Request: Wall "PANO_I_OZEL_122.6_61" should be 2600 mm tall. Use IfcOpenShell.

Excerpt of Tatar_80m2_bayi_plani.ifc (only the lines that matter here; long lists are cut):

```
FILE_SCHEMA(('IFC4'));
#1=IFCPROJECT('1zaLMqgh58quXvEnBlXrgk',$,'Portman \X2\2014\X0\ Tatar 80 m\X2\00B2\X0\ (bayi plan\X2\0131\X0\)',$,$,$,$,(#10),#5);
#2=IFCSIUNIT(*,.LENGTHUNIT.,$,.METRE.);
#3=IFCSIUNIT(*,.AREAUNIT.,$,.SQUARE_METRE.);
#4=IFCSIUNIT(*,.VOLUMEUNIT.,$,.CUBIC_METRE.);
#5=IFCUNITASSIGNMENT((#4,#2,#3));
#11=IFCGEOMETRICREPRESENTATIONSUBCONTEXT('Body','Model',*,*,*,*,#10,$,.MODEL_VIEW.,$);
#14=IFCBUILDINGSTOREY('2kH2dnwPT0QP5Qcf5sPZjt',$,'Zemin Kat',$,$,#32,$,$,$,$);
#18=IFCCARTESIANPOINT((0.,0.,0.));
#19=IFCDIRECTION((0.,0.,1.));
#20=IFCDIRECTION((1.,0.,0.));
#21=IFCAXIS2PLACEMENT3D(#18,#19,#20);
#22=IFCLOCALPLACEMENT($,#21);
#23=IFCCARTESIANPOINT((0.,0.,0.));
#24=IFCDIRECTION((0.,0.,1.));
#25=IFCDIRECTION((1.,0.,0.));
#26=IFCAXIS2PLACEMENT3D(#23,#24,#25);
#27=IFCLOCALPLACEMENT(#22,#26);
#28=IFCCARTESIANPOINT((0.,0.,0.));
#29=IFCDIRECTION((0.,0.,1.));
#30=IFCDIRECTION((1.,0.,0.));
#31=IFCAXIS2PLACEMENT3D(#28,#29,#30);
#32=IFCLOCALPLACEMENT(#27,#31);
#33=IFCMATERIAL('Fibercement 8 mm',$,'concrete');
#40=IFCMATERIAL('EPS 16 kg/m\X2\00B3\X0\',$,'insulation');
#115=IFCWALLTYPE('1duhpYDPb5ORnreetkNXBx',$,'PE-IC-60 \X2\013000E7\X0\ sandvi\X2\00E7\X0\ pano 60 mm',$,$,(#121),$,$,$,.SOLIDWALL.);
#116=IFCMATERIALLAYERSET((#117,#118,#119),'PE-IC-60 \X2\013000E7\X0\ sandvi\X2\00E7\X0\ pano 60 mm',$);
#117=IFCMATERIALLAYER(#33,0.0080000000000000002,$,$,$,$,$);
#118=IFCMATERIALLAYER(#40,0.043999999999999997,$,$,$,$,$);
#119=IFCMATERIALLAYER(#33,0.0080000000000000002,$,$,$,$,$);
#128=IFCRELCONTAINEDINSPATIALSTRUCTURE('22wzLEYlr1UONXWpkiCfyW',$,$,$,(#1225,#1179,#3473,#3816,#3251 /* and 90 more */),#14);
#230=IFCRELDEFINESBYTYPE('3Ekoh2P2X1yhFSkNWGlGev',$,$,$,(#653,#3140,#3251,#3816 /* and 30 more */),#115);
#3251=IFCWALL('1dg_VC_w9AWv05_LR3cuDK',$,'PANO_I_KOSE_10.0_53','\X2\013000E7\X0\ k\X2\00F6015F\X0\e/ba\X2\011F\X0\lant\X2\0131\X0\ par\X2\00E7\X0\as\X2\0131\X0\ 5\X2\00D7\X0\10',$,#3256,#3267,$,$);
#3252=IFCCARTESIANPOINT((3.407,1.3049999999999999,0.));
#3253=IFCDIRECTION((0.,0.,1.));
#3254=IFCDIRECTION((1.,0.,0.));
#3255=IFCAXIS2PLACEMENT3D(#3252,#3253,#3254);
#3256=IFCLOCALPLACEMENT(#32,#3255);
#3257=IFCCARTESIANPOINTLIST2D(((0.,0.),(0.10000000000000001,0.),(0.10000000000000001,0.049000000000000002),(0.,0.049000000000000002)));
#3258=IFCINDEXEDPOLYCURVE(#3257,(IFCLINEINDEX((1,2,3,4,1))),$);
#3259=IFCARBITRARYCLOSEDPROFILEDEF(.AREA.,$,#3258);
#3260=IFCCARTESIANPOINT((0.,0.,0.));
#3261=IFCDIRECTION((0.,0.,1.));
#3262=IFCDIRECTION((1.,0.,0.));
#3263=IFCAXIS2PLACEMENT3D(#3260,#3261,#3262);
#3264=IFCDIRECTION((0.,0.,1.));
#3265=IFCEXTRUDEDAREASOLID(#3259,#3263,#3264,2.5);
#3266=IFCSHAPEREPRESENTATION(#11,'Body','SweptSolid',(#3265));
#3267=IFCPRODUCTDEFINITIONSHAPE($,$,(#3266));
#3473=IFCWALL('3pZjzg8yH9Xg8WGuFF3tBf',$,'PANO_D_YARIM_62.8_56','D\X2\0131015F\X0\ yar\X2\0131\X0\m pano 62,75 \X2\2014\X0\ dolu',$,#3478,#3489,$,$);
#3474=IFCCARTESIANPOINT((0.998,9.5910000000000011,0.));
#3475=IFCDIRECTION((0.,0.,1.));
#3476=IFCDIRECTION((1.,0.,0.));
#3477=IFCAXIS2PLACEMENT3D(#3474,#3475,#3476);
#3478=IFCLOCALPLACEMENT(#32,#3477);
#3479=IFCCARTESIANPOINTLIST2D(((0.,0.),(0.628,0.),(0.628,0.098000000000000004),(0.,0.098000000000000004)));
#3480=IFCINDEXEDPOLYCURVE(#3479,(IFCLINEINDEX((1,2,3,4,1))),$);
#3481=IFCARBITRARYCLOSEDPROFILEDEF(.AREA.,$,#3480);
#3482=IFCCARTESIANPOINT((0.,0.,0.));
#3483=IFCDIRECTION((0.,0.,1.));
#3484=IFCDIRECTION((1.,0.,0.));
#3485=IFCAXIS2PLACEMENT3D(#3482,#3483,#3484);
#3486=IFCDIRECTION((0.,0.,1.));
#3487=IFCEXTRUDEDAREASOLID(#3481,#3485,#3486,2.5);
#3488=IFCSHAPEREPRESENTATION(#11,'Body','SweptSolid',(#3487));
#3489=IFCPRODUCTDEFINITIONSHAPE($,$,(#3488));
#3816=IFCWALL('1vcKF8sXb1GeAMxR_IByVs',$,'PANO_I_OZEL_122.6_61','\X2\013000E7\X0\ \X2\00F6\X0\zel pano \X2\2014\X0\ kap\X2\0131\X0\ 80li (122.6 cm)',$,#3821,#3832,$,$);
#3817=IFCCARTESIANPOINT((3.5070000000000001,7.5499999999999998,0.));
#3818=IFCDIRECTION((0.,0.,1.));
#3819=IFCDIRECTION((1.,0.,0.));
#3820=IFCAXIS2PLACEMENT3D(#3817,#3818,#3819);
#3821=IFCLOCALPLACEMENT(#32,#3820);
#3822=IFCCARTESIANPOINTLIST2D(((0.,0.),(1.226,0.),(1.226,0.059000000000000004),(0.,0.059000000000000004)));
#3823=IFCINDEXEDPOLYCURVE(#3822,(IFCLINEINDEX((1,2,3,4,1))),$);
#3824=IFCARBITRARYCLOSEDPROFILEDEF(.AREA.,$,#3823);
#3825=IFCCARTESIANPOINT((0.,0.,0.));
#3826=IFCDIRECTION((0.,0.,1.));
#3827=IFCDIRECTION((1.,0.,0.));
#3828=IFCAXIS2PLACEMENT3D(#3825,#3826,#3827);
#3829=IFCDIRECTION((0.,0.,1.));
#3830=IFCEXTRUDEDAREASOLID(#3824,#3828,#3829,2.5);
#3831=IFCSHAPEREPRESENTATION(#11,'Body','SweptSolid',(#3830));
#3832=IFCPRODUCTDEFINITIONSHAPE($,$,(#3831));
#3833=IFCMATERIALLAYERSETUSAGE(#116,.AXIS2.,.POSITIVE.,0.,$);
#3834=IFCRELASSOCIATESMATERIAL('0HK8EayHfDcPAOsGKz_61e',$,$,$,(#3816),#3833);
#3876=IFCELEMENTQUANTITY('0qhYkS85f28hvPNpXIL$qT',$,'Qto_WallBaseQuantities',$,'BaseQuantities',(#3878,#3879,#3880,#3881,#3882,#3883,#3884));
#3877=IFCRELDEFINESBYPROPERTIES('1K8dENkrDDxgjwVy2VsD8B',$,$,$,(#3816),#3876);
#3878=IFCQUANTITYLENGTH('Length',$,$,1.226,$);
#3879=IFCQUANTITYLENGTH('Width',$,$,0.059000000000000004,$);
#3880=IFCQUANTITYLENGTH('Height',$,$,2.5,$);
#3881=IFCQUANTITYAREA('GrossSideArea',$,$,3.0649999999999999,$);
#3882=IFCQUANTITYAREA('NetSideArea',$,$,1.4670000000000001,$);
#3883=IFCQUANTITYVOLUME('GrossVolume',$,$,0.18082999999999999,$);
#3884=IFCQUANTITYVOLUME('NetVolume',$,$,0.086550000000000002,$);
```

```python
import ifcopenshell
import ifcopenshell.api.pset
import ifcopenshell.geom
import ifcopenshell.util.element
import ifcopenshell.util.representation
import ifcopenshell.util.shape
import ifcopenshell.util.unit

model = ifcopenshell.open("Tatar_80m2_bayi_plani.ifc")
unit_scale = ifcopenshell.util.unit.calculate_unit_scale(model)
area_scale = ifcopenshell.util.unit.calculate_unit_scale(model, "AREAUNIT")
volume_scale = ifcopenshell.util.unit.calculate_unit_scale(model, "VOLUMEUNIT")
settings = ifcopenshell.geom.settings()


def volume(element):
    """Net volume in cubic metres, openings subtracted."""
    shape = ifcopenshell.geom.create_shape(settings, element)
    return ifcopenshell.util.shape.get_volume(shape.geometry)


wall = model.by_id(3816)
before = volume(wall)

body = ifcopenshell.util.representation.get_representation(wall, "Model", "Body")
solid = body.Items[0]
old_height = solid.Depth
solid.Depth = 2.6 / unit_scale
after = volume(wall)
thickness = 0.059  # wall thickness in metres

# Update the stored height, areas and volumes.
qto = model.by_id(ifcopenshell.util.element.get_pset(wall, "Qto_WallBaseQuantities", should_inherit=False)["id"])
ifcopenshell.api.pset.edit_qto(model, qto=qto, properties={
    "Height": solid.Depth,
    "GrossSideArea": ifcopenshell.util.element.get_pset(wall, "Qto_WallBaseQuantities", "GrossSideArea") * solid.Depth / old_height,
    "NetSideArea": after / thickness / area_scale,
    "GrossVolume": ifcopenshell.util.element.get_pset(wall, "Qto_WallBaseQuantities", "GrossVolume") * solid.Depth / old_height,
    "NetVolume": after / volume_scale,
})

print(f"height {old_height:g} -> {solid.Depth:g}, volume {before:.3f} -> {after:.3f} m3")

model.write("Tatar_80m2_bayi_plani_v2.ifc")
```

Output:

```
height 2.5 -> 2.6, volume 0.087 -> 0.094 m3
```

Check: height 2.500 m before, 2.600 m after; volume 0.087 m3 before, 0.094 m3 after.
